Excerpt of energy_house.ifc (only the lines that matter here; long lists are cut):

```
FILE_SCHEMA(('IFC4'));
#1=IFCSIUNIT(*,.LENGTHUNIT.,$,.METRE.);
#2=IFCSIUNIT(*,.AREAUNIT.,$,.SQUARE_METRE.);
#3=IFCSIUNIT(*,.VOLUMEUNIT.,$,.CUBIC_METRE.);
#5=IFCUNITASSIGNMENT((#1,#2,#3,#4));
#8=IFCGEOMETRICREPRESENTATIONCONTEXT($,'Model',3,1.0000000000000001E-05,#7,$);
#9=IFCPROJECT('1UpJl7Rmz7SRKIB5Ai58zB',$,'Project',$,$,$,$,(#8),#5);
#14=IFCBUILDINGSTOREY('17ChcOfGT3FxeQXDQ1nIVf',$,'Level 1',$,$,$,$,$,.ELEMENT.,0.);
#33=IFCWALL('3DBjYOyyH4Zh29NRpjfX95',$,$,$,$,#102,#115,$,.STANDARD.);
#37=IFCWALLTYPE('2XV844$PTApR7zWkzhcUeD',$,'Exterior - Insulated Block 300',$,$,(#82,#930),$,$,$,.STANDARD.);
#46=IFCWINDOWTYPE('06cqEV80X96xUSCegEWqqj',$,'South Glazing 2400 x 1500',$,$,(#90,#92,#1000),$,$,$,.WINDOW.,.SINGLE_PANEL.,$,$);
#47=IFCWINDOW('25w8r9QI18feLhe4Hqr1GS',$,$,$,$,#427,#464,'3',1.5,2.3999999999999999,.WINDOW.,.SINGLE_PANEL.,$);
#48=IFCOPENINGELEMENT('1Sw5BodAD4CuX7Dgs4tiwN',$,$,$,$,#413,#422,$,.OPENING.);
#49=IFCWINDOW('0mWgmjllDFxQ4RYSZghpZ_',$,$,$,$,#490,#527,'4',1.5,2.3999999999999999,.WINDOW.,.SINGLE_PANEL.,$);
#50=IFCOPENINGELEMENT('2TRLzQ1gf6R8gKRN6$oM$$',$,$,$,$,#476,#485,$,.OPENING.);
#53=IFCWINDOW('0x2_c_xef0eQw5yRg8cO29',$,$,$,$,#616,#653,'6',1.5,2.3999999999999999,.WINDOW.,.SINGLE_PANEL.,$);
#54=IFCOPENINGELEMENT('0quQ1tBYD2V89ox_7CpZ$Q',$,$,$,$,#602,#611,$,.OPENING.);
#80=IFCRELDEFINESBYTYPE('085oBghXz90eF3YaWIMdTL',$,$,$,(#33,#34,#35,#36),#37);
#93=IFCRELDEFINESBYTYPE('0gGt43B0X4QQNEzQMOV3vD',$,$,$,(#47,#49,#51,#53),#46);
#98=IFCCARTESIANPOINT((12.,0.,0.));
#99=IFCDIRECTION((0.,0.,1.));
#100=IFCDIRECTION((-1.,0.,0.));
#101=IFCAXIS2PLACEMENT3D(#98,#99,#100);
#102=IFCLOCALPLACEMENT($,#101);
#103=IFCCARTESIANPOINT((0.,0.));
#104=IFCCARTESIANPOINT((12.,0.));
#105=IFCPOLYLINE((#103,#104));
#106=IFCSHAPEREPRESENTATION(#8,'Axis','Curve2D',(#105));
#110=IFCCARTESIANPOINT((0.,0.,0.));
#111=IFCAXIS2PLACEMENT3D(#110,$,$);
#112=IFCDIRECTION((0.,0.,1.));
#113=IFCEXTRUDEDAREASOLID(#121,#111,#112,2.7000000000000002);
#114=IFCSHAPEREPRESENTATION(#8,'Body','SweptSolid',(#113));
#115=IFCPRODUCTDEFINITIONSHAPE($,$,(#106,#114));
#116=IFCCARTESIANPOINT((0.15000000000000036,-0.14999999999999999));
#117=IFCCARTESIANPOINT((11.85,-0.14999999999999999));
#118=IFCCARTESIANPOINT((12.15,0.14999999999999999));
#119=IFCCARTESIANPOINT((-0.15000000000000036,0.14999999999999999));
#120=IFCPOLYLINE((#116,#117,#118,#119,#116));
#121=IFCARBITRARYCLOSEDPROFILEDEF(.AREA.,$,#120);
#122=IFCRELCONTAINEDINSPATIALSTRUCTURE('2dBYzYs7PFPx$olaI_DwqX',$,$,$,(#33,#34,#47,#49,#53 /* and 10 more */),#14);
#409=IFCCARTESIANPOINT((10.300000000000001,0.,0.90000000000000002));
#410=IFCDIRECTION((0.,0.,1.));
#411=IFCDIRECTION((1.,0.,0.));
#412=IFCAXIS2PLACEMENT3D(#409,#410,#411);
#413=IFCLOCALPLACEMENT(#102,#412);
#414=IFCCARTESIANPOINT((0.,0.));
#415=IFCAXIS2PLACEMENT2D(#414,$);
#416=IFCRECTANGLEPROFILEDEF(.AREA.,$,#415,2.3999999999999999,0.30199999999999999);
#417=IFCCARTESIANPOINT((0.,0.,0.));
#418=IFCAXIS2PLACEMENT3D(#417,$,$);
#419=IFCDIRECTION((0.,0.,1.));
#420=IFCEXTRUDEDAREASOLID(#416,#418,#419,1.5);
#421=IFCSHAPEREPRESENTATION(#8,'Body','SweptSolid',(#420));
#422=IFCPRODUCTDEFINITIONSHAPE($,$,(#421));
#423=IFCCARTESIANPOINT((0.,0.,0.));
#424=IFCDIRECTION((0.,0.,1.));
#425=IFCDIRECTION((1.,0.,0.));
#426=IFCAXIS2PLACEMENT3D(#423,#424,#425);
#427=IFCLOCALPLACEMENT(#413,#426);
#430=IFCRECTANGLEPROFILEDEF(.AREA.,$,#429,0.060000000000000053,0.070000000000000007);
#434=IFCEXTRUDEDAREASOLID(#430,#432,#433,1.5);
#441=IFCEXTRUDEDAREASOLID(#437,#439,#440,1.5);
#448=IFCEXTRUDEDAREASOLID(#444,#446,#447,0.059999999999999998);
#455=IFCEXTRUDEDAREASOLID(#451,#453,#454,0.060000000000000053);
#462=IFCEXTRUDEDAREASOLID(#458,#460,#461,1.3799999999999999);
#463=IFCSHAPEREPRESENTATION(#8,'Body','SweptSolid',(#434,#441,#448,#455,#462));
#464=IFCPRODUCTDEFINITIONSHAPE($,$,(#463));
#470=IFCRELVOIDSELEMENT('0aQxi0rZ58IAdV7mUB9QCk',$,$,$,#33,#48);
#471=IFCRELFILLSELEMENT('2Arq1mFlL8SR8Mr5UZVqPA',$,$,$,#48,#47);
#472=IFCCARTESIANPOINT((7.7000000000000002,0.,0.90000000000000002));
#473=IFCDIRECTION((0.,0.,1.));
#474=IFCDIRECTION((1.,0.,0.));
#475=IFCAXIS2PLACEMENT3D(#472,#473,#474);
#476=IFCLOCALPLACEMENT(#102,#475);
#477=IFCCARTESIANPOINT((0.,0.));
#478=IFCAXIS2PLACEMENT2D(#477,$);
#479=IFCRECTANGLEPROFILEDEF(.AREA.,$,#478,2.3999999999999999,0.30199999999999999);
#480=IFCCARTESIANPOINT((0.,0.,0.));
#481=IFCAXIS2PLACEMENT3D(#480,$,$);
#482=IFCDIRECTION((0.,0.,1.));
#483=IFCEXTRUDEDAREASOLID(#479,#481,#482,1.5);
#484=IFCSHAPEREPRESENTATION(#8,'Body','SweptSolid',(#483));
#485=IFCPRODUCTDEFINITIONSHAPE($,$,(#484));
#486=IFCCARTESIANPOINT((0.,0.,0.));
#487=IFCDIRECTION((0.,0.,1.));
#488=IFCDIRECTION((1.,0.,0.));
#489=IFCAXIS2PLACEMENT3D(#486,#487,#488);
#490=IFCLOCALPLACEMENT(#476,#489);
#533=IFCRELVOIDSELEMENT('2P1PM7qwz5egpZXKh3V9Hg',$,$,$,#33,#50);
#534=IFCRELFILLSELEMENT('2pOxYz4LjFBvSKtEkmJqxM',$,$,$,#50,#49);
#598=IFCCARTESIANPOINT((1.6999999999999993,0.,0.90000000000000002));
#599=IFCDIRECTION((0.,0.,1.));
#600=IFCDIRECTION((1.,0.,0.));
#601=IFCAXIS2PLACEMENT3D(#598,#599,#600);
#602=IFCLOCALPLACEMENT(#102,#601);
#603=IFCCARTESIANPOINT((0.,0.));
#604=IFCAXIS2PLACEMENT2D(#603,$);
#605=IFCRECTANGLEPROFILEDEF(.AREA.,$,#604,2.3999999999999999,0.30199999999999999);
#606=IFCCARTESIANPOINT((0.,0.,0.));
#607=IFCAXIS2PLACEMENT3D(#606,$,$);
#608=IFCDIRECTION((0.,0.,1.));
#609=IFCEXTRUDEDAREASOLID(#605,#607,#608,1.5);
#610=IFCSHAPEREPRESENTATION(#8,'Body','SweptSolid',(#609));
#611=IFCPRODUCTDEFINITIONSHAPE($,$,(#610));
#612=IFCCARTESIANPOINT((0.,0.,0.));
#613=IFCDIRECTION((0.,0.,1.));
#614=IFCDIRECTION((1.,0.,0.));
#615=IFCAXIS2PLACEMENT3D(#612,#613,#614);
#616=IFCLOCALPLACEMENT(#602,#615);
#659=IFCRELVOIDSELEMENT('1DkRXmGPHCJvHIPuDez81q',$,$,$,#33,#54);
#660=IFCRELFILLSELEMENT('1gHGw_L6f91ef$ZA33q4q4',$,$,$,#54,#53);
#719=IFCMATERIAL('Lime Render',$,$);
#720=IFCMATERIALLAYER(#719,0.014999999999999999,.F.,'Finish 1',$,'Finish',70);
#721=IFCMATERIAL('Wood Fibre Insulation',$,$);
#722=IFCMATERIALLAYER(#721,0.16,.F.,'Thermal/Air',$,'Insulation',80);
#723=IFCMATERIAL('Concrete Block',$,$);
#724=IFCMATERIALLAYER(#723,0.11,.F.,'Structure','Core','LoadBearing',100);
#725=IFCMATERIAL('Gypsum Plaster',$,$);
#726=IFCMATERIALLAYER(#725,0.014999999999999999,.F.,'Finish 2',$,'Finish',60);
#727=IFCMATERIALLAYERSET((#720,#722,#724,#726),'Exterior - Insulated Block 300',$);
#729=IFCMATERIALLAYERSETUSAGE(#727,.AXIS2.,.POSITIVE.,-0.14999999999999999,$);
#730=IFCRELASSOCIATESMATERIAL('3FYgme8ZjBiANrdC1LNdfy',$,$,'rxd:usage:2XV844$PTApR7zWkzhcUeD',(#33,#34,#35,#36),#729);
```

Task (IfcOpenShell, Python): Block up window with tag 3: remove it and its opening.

```python
import ifcopenshell
import ifcopenshell.api.feature
import ifcopenshell.api.root
import ifcopenshell.geom
import ifcopenshell.util.shape

model = ifcopenshell.open("energy_house.ifc")
settings = ifcopenshell.geom.settings()


def volume(element):
    """Net volume in cubic metres, openings subtracted."""
    shape = ifcopenshell.geom.create_shape(settings, element)
    return ifcopenshell.util.shape.get_volume(shape.geometry)


window = model.by_guid("25w8r9QI18feLhe4Hqr1GS")
opening = window.FillsVoids[0].RelatingOpeningElement
wall = opening.VoidsElements[0].RelatingBuildingElement
before = volume(wall)

ifcopenshell.api.root.remove_product(model, product=window)
ifcopenshell.api.feature.remove_feature(model, feature=opening)

after = volume(wall)

print(f"wall volume {before:.3f} -> {after:.3f} m3")

model.write("energy_house-out.ifc")
```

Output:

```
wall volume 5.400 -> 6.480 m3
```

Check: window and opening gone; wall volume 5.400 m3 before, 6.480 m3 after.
